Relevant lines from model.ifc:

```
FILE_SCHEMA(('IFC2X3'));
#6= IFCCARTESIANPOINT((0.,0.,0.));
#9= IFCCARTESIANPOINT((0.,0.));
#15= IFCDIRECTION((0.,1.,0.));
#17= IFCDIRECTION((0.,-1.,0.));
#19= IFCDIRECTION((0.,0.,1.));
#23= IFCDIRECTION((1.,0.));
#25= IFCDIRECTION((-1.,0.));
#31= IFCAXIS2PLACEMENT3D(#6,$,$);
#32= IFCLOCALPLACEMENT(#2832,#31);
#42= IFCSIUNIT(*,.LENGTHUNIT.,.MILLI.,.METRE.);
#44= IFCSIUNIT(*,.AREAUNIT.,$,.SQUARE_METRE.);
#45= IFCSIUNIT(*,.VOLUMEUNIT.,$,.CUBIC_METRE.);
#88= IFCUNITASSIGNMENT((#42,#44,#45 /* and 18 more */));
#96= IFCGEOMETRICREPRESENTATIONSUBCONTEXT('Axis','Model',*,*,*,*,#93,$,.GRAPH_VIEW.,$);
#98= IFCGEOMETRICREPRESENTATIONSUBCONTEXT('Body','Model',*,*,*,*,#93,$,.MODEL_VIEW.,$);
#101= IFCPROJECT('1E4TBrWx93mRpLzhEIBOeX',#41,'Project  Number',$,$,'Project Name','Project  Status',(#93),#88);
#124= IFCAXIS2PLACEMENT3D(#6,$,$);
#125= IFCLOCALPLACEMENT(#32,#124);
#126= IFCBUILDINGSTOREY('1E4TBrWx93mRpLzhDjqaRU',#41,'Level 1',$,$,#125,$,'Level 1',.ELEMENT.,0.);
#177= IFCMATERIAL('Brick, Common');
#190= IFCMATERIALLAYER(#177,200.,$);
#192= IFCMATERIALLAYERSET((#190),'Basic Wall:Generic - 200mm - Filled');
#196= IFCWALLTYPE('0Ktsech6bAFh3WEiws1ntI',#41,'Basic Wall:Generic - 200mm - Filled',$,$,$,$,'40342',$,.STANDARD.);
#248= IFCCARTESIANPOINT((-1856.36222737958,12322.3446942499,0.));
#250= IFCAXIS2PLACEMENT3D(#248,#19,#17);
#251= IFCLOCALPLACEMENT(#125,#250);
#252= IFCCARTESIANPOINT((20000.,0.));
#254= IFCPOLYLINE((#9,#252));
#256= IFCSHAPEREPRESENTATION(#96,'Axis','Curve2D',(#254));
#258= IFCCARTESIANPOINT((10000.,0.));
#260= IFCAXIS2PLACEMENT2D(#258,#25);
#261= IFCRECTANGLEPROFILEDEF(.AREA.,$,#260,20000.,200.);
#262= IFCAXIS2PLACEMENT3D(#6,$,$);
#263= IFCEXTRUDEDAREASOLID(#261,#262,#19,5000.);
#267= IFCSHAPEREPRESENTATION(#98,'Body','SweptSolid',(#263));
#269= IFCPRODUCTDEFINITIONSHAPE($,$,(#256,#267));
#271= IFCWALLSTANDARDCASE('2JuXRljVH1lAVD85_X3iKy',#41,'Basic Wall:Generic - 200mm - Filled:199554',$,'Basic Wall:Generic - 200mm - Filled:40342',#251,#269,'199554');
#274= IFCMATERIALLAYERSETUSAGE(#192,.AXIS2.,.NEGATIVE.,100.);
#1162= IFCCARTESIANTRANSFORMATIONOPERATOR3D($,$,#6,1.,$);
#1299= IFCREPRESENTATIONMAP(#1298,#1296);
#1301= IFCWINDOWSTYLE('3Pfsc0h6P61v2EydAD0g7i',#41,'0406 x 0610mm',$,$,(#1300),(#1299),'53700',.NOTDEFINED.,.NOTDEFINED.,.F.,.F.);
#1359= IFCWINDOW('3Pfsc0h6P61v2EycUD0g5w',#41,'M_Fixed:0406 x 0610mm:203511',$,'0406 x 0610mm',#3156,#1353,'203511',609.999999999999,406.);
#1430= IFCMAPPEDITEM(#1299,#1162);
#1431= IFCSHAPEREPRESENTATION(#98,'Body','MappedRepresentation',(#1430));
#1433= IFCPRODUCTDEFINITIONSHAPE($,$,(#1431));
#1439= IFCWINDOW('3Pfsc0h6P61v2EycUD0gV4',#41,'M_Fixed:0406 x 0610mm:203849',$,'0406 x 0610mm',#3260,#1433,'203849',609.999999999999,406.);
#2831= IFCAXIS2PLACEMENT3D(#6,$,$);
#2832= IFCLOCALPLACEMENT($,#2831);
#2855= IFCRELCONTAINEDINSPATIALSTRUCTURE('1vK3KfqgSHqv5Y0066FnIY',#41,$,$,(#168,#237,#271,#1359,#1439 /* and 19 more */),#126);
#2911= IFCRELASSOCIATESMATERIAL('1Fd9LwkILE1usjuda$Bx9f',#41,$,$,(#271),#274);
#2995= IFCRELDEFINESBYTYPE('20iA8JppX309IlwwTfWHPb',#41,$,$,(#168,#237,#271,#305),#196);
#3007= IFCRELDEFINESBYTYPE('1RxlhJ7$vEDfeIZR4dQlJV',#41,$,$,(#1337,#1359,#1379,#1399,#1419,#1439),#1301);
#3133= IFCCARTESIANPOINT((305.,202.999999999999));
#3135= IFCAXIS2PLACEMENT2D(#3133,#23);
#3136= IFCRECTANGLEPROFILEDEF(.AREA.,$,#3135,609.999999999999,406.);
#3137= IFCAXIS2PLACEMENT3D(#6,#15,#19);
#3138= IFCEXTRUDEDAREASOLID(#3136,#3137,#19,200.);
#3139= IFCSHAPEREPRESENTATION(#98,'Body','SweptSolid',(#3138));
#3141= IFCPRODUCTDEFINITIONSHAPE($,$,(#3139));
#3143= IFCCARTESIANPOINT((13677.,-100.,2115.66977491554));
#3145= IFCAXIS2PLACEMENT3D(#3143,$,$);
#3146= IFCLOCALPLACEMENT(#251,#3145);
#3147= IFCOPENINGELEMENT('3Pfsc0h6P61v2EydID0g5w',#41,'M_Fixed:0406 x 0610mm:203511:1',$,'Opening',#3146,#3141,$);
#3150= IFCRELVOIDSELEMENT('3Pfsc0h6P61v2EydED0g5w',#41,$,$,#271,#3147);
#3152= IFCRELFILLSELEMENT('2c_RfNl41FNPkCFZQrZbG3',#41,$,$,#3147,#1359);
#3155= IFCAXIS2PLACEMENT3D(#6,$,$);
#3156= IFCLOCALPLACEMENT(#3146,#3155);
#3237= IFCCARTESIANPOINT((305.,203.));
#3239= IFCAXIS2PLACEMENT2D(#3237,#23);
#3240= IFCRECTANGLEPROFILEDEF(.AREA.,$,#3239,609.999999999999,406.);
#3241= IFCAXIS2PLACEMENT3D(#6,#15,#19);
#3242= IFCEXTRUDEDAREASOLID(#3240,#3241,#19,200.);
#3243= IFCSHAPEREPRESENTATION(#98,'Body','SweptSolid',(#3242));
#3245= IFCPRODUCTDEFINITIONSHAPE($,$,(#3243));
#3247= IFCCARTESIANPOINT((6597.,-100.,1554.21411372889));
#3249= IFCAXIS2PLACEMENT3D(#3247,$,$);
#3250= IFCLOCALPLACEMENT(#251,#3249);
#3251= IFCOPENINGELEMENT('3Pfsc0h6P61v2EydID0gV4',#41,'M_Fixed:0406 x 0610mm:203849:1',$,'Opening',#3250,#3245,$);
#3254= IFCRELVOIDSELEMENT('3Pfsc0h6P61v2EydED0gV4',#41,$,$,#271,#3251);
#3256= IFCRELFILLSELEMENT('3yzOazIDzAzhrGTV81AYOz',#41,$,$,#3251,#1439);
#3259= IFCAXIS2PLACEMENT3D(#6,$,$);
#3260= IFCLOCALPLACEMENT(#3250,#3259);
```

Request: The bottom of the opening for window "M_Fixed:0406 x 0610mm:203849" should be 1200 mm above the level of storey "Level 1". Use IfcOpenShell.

```python
import numpy as np
import ifcopenshell
import ifcopenshell.api.geometry
import ifcopenshell.geom
import ifcopenshell.util.element
import ifcopenshell.util.placement
import ifcopenshell.util.shape
import ifcopenshell.util.unit

model = ifcopenshell.open("model.ifc")
unit_scale = ifcopenshell.util.unit.calculate_unit_scale(model)

window = model.by_guid("3Pfsc0h6P61v2EycUD0gV4")
opening = window.FillsVoids[0].RelatingOpeningElement
storey = ifcopenshell.util.element.get_container(window, ifc_class="IfcBuildingStorey")
level = ifcopenshell.util.placement.get_local_placement(storey.ObjectPlacement)[2, 3]

# The opening's origin need not be at the sill, so measure its lowest point.
shape = ifcopenshell.geom.create_shape(ifcopenshell.geom.settings(), opening)
bottom = ifcopenshell.util.shape.get_shape_bottom_elevation(shape, shape.geometry) / unit_scale
dz = level + 1200.0 - bottom

shift = np.array([0.0, 0.0, dz])
# The window is placed relative to its opening, so it follows when the opening moves.
matrix = ifcopenshell.util.placement.get_local_placement(opening.ObjectPlacement)
matrix[:3, 3] += shift
ifcopenshell.api.geometry.edit_object_placement(
    model, product=opening, matrix=matrix, is_si=False, should_transform_children=True
)

print(f"moved by {dz * unit_scale:+.3f} m")

model.write("model-out.ifc")
```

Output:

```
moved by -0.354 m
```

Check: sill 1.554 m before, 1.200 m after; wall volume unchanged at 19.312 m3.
